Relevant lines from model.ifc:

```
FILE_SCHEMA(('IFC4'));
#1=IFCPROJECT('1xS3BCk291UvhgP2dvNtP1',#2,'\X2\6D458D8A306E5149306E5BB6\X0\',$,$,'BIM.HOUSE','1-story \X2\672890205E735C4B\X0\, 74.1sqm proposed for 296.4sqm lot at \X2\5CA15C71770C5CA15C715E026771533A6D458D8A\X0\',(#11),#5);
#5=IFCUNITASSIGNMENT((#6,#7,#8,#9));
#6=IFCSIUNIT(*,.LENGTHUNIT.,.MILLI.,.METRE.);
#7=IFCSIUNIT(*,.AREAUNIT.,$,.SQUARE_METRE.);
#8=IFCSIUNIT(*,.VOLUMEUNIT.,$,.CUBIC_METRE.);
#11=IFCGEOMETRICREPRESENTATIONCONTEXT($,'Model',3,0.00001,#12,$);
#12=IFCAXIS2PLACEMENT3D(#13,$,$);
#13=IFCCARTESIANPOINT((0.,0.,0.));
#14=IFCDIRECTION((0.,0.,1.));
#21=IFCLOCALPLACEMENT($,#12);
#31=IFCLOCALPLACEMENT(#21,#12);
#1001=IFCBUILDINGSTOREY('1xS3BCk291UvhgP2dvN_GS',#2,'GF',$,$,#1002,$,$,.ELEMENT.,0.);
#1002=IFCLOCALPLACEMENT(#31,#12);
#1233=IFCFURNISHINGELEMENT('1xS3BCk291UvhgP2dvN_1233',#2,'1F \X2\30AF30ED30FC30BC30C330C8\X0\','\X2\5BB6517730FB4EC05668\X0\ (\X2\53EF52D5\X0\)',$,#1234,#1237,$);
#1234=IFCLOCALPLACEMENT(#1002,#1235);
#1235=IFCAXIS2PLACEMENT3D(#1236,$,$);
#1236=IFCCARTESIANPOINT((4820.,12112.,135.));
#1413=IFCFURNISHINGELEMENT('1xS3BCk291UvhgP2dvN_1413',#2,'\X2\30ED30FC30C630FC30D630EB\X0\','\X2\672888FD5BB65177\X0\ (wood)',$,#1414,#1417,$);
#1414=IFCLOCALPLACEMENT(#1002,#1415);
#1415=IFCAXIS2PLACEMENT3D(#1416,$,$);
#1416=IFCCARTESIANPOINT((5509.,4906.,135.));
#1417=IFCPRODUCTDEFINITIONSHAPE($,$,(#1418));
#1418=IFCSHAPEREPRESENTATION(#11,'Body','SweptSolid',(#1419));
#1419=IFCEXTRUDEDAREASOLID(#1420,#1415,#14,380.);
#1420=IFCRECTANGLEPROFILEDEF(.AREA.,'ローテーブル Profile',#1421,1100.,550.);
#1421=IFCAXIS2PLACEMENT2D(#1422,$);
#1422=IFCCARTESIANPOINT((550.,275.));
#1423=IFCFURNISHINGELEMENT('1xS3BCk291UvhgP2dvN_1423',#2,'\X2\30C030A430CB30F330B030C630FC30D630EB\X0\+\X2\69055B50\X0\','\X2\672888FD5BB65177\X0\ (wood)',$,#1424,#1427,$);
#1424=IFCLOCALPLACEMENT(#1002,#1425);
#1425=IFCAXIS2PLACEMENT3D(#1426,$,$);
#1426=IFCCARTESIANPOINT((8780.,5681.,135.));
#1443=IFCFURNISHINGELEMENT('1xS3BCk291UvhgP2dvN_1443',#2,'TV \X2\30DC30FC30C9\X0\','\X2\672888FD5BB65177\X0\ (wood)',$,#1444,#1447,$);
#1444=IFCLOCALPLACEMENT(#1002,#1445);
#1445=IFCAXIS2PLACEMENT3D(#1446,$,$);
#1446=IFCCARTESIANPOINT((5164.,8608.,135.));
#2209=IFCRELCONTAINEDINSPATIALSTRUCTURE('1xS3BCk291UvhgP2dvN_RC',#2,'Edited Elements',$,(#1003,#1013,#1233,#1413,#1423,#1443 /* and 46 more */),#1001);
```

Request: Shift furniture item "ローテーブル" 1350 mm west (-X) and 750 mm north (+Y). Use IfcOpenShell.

```python
import ifcopenshell
import ifcopenshell.api.geometry
import ifcopenshell.util.placement
import ifcopenshell.util.unit

model = ifcopenshell.open("model.ifc")
unit_scale = ifcopenshell.util.unit.calculate_unit_scale(model)

item = model.by_guid("1xS3BCk291UvhgP2dvN_1413")
matrix = ifcopenshell.util.placement.get_local_placement(item.ObjectPlacement)
matrix[0, 3] -= 1.35 / unit_scale
matrix[1, 3] += 0.75 / unit_scale
ifcopenshell.api.geometry.edit_object_placement(model, product=item, matrix=matrix, is_si=False)

print(ifcopenshell.util.placement.get_local_placement(item.ObjectPlacement).round(3) + 0.0)

model.write("model_updated.ifc")
```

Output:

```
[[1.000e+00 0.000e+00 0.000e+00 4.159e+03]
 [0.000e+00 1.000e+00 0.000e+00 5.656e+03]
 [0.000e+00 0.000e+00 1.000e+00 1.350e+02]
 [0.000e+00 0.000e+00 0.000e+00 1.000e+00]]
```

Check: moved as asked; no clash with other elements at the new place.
